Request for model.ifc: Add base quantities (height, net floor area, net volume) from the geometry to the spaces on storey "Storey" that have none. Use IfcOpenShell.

First a look at what the model holds.

```python
import ifcopenshell
import ifcopenshell.util.element
import ifcopenshell.util.unit

model = ifcopenshell.open("model.ifc")
print(model.schema)
for unit_type in ("LENGTHUNIT", "AREAUNIT", "VOLUMEUNIT"):
    print(unit_type, ifcopenshell.util.unit.calculate_unit_scale(model, unit_type))
storey = next(s for s in model.by_type("IfcBuildingStorey") if s.Name == "Storey")
spaces = [e for e in ifcopenshell.util.element.get_decomposition(storey) if e.is_a("IfcSpace")]
for e in sorted(spaces, key=lambda e: e.id()):
    print(e.id(), e.is_a(), e.Name, list(ifcopenshell.util.element.get_psets(e, qtos_only=True)), sep=" | ")
```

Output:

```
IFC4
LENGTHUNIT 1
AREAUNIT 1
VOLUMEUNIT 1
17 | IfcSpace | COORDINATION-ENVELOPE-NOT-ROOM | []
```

```python
import ifcopenshell
import ifcopenshell.api.pset
import ifcopenshell.geom
import ifcopenshell.util.element
import ifcopenshell.util.shape
import ifcopenshell.util.unit

model = ifcopenshell.open("model.ifc")
unit_scale = ifcopenshell.util.unit.calculate_unit_scale(model)
area_scale = ifcopenshell.util.unit.calculate_unit_scale(model, "AREAUNIT")
volume_scale = ifcopenshell.util.unit.calculate_unit_scale(model, "VOLUMEUNIT")
settings = ifcopenshell.geom.settings()

storey = next(s for s in model.by_type("IfcBuildingStorey") if s.Name == "Storey")
spaces = [e for e in ifcopenshell.util.element.get_decomposition(storey) if e.is_a("IfcSpace")]

for e in sorted(spaces, key=lambda e: e.id()):
    if ifcopenshell.util.element.get_psets(e, qtos_only=True, should_inherit=False):
        continue
    # Geometry comes back in metres, in the element's own axes.
    shape = ifcopenshell.geom.create_shape(settings, e)
    values = {
        "Height": ifcopenshell.util.shape.get_z(shape.geometry) / unit_scale,
        "NetFloorArea": ifcopenshell.util.shape.get_footprint_area(shape.geometry) / area_scale,
        "NetVolume": ifcopenshell.util.shape.get_volume(shape.geometry) / volume_scale,
    }
    qto = ifcopenshell.api.pset.add_qto(model, product=e, name="Qto_SpaceBaseQuantities")
    ifcopenshell.api.pset.edit_qto(model, qto=qto, properties=values)
    print(e.id(), {k: round(v, 3) for k, v in values.items()})

model.write("model_edited.ifc")
```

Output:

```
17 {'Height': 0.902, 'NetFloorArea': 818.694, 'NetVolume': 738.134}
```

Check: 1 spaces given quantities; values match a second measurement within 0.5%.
